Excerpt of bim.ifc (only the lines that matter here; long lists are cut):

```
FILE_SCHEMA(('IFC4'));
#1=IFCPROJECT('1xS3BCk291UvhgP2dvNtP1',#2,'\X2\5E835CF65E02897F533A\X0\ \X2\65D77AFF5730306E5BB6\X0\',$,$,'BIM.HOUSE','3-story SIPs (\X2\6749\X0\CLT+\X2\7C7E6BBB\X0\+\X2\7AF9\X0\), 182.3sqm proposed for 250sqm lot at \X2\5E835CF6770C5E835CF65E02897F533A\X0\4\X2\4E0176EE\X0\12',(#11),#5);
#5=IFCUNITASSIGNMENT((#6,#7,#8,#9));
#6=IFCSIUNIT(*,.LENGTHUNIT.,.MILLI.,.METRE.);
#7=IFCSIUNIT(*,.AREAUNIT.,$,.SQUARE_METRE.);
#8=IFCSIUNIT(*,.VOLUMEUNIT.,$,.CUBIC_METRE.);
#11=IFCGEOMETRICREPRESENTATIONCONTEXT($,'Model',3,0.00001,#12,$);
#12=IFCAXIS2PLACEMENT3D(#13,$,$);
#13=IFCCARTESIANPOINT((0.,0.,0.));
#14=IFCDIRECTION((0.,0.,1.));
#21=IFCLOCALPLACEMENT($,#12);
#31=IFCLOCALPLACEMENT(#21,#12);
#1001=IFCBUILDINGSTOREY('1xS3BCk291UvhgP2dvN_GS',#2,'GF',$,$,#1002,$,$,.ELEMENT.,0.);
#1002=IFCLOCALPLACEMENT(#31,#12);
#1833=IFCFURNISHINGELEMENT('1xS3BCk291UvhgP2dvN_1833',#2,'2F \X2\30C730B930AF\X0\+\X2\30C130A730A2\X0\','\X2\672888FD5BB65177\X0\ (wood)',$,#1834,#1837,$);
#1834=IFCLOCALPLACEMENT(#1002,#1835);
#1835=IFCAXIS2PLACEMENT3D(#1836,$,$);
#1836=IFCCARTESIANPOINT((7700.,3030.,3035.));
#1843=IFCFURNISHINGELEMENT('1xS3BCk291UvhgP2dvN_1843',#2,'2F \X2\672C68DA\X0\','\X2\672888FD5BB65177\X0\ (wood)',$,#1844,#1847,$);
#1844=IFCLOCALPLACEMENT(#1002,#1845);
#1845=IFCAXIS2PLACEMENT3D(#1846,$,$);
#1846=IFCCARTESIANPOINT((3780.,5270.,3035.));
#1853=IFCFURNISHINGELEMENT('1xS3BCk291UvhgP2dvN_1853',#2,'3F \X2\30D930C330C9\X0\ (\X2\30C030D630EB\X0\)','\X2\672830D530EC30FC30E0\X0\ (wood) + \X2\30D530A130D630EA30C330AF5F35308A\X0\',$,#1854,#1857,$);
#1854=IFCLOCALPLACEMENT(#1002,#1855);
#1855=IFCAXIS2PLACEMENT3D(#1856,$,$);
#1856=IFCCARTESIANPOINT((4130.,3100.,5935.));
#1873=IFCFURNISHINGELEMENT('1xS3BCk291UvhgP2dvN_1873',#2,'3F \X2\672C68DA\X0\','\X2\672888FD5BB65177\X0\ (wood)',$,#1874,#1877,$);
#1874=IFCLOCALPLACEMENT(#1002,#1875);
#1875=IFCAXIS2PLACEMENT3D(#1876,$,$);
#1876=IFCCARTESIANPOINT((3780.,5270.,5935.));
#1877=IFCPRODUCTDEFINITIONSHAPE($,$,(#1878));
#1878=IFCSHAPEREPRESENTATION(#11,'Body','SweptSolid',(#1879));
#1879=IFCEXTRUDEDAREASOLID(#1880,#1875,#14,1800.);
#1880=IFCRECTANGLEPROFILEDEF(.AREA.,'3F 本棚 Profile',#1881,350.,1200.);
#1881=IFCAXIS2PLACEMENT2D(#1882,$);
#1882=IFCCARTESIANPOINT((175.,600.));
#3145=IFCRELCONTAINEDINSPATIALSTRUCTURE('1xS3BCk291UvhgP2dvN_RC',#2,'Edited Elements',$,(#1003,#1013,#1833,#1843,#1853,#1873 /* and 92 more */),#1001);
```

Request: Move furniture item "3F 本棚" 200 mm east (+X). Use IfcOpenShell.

```python
import ifcopenshell
import ifcopenshell.api.geometry
import ifcopenshell.util.placement
import ifcopenshell.util.unit

model = ifcopenshell.open("bim.ifc")
unit_scale = ifcopenshell.util.unit.calculate_unit_scale(model)

item = model.by_id(1873)
matrix = ifcopenshell.util.placement.get_local_placement(item.ObjectPlacement)
matrix[0, 3] += 0.2 / unit_scale
ifcopenshell.api.geometry.edit_object_placement(model, product=item, matrix=matrix, is_si=False)

print(ifcopenshell.util.placement.get_local_placement(item.ObjectPlacement).round(3) + 0.0)

model.write("bim-out.ifc")
```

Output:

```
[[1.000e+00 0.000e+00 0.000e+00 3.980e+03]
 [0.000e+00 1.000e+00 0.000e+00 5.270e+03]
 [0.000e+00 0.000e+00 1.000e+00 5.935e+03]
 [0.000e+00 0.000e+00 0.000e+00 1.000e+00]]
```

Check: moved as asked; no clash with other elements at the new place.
